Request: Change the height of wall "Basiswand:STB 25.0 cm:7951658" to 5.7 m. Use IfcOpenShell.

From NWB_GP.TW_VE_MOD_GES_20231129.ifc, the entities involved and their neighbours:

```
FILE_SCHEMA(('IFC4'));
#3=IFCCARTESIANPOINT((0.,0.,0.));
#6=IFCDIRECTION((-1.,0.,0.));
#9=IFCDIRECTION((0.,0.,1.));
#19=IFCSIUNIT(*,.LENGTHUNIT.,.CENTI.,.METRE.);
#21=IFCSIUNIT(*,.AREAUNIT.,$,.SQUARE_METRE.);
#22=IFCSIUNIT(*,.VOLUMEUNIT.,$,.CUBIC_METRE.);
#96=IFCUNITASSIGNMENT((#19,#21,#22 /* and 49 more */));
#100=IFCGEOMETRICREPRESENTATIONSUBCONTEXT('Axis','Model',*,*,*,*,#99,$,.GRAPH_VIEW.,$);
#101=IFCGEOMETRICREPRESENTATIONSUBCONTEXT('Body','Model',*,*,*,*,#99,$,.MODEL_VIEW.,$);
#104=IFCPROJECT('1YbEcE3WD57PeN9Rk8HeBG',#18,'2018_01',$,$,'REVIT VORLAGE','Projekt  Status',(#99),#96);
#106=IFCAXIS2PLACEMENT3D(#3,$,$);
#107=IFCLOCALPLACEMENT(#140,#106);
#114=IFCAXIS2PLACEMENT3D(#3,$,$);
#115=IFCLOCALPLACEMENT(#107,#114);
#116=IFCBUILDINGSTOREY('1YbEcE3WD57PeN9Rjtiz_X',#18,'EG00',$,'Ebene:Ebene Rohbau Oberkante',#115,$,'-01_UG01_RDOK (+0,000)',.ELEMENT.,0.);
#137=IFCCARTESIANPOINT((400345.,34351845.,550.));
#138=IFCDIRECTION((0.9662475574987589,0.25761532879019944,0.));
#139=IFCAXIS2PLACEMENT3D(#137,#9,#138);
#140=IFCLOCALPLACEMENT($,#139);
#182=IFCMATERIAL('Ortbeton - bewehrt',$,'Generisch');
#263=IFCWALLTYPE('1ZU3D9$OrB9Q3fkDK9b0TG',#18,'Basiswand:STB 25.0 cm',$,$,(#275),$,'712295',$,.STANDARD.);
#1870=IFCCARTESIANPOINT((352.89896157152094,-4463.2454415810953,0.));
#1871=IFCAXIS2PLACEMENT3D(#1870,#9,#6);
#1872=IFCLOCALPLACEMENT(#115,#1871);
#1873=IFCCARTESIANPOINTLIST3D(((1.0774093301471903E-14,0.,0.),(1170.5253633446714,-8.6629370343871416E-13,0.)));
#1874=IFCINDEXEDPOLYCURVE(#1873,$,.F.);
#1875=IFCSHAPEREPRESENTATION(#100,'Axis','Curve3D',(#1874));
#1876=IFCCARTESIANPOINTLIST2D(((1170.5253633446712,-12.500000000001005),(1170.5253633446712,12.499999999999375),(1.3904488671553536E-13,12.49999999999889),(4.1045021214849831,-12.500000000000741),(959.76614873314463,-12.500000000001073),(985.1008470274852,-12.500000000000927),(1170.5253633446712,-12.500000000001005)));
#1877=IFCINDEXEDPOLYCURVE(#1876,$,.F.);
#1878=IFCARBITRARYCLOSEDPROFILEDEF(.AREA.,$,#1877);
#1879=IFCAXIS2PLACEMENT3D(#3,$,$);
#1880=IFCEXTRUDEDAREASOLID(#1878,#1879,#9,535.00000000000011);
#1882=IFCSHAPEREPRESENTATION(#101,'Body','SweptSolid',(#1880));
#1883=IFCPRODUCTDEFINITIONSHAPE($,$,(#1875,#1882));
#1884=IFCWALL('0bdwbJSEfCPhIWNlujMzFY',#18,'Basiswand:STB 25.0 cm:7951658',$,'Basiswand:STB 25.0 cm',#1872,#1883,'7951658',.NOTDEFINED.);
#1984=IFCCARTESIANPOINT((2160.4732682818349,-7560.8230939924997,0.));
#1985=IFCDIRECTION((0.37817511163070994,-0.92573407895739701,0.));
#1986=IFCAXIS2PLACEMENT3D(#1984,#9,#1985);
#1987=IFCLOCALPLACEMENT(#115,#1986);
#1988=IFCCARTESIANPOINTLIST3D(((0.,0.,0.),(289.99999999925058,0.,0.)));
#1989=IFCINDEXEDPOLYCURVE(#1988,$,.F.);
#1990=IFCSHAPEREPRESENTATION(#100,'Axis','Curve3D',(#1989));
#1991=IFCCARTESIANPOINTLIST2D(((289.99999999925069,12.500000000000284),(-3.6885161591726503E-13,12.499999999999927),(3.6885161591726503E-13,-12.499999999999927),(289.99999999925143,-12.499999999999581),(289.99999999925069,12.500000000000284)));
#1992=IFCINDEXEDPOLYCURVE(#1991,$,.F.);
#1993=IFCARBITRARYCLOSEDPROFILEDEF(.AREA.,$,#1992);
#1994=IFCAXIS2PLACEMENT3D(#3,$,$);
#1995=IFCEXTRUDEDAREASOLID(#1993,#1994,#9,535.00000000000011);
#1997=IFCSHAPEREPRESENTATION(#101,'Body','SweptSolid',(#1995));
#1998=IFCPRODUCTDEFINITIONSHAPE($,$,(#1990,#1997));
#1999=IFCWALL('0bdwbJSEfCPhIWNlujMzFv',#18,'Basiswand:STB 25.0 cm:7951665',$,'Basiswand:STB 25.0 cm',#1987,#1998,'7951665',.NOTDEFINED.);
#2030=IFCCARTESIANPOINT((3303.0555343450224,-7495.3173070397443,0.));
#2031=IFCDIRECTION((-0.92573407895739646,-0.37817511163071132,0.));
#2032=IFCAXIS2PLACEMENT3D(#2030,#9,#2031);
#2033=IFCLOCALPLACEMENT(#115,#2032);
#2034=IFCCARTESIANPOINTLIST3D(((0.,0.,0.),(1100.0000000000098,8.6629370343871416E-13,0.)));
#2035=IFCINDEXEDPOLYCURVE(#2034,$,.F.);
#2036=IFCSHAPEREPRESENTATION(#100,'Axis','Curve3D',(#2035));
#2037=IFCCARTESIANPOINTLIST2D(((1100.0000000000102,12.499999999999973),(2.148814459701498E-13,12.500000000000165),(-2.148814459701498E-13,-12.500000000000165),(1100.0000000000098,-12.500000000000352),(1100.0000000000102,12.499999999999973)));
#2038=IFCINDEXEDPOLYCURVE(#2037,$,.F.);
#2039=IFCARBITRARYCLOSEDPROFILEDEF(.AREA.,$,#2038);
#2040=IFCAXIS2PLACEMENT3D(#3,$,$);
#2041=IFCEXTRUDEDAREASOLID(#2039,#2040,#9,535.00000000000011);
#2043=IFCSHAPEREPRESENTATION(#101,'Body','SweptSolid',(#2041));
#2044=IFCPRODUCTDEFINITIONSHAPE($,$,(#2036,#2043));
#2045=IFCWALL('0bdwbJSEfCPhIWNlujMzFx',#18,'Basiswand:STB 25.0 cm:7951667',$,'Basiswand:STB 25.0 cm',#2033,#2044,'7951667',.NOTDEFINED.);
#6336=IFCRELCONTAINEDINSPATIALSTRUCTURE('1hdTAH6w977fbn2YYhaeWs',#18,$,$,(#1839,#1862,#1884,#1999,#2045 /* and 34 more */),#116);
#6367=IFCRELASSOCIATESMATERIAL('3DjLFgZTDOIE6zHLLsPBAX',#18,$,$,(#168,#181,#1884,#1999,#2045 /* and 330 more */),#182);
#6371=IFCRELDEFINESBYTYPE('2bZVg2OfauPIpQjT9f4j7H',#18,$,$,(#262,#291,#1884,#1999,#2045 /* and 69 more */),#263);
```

```python
import ifcopenshell
import ifcopenshell.geom
import ifcopenshell.util.representation
import ifcopenshell.util.shape
import ifcopenshell.util.unit

model = ifcopenshell.open("NWB_GP.TW_VE_MOD_GES_20231129.ifc")
unit_scale = ifcopenshell.util.unit.calculate_unit_scale(model)
settings = ifcopenshell.geom.settings()


def volume(element):
    """Net volume in cubic metres, openings subtracted."""
    shape = ifcopenshell.geom.create_shape(settings, element)
    return ifcopenshell.util.shape.get_volume(shape.geometry)


wall = model.by_id(1884)
before = volume(wall)

body = ifcopenshell.util.representation.get_representation(wall, "Model", "Body")
solid = body.Items[0]
old_height = solid.Depth
solid.Depth = 5.7 / unit_scale
after = volume(wall)

print(f"height {old_height:g} -> {solid.Depth:g}, volume {before:.3f} -> {after:.3f} m3")

model.write("NWB_GP.TW_VE_MOD_GES_20231129_rev.ifc")
```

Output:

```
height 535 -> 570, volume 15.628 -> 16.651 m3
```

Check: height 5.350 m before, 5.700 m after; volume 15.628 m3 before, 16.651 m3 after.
